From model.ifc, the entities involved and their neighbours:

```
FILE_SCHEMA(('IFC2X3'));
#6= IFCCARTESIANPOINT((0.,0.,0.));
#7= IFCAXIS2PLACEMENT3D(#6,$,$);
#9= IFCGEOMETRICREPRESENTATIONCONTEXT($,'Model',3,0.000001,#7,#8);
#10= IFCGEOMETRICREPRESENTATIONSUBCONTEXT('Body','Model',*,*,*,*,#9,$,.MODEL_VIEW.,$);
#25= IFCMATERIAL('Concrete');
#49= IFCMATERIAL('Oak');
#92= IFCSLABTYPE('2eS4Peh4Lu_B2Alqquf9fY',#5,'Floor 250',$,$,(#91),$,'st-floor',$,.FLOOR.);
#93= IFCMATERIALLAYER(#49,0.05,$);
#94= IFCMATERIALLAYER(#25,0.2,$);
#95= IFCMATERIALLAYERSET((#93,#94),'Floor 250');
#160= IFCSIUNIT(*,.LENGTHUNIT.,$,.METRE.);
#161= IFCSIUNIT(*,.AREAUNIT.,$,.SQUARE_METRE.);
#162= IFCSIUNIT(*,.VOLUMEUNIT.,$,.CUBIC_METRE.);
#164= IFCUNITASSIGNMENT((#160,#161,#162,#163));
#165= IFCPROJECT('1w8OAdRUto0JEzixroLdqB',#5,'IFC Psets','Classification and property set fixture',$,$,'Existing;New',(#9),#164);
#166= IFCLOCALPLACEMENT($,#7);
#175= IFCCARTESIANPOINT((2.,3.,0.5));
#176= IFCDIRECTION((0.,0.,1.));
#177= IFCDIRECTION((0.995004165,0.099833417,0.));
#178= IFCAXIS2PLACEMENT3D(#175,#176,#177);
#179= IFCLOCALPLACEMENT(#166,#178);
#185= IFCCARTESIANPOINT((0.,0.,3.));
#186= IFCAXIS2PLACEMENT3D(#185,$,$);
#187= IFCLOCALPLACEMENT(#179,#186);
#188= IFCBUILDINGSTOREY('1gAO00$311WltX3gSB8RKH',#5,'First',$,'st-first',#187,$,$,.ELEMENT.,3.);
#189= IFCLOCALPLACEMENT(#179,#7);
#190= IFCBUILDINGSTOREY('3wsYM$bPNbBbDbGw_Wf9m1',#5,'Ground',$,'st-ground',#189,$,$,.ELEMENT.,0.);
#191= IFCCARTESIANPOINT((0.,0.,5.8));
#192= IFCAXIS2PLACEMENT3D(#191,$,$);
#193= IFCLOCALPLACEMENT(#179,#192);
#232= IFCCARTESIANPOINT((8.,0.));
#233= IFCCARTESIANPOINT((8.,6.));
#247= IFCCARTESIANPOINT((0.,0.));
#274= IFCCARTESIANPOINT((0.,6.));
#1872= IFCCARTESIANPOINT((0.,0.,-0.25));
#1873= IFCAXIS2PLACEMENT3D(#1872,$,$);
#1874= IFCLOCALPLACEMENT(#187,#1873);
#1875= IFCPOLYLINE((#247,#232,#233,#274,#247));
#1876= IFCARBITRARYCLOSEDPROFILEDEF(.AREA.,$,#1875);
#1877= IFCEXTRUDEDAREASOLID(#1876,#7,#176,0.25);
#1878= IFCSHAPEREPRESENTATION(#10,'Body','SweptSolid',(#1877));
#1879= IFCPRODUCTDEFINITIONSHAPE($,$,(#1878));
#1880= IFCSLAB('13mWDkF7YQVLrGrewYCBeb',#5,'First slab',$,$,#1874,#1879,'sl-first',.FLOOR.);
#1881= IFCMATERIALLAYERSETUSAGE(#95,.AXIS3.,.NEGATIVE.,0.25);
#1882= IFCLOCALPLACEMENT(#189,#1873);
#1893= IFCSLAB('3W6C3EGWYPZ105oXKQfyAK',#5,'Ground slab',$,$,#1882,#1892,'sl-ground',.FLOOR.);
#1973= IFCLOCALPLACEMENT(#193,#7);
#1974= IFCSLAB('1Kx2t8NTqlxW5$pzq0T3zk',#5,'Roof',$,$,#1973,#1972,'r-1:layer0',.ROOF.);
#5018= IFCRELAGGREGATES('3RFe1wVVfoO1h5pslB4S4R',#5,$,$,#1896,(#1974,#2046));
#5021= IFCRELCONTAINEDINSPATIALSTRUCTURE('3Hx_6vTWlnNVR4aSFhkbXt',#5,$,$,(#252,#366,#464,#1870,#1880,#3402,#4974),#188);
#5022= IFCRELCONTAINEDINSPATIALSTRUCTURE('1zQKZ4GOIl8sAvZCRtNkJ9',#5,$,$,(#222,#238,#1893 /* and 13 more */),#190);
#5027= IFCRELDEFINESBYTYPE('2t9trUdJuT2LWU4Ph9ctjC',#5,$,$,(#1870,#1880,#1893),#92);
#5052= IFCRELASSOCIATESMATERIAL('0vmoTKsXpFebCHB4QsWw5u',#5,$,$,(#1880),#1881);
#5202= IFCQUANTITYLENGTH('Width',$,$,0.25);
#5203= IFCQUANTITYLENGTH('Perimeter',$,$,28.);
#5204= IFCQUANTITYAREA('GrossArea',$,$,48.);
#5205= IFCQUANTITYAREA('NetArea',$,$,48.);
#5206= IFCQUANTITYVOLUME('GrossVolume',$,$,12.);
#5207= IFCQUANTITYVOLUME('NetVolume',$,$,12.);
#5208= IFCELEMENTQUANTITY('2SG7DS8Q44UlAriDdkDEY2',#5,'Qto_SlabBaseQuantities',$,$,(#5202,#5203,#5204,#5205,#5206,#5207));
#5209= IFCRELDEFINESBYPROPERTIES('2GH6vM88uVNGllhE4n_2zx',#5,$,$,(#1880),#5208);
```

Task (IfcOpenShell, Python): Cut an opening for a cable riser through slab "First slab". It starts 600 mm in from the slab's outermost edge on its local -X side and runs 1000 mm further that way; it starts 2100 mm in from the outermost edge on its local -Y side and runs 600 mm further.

```python
import numpy as np
import ifcopenshell
import ifcopenshell.api.feature
import ifcopenshell.api.geometry
import ifcopenshell.api.pset
import ifcopenshell.api.root
import ifcopenshell.geom
import ifcopenshell.util.element
import ifcopenshell.util.placement
import ifcopenshell.util.representation
import ifcopenshell.util.shape
import ifcopenshell.util.unit

model = ifcopenshell.open("model.ifc")
unit_scale = ifcopenshell.util.unit.calculate_unit_scale(model)
area_scale = ifcopenshell.util.unit.calculate_unit_scale(model, "AREAUNIT")
volume_scale = ifcopenshell.util.unit.calculate_unit_scale(model, "VOLUMEUNIT")
settings = ifcopenshell.geom.settings()


def volume(element):
    """Net volume in cubic metres, openings subtracted."""
    shape = ifcopenshell.geom.create_shape(settings, element)
    return ifcopenshell.util.shape.get_volume(shape.geometry)


slab = model.by_id(1880)
before = volume(slab)

# Extent in the slab's own axes, in metres. The edges named are its -X and -Y sides.
slab_shape = ifcopenshell.geom.create_shape(settings, slab)
vertices = ifcopenshell.util.shape.get_vertices(slab_shape.geometry)
x_min, y_min, bottom = vertices.min(axis=0)
top = vertices[:, 2].max()

opening = ifcopenshell.api.root.create_entity(model, ifc_class="IfcOpeningElement", name="Cable riser opening")
context = ifcopenshell.util.representation.get_context(model, "Model", "Body", "MODEL_VIEW")
width, depth = 1, 0.6
outline = [(0.0, 0.0), (width, 0.0), (width, depth), (0.0, depth), (0.0, 0.0)]
# Overshoot both faces by 50 mm so the cut is clean.
shape = ifcopenshell.api.geometry.add_slab_representation(
    model, context=context, depth=top - bottom + 0.1, polyline=outline
)
ifcopenshell.api.geometry.assign_representation(model, product=opening, representation=shape)

matrix = ifcopenshell.util.placement.get_local_placement(slab.ObjectPlacement)
matrix[:, 3] = matrix @ np.append(np.array([x_min + 0.6, y_min + 2.1, bottom - 0.05]) / unit_scale, 1.0)
ifcopenshell.api.geometry.edit_object_placement(model, product=opening, matrix=matrix, is_si=False)
ifcopenshell.api.feature.add_feature(model, feature=opening, element=slab)

after = volume(slab)

# Update the slab's stored quantities.
qto = model.by_id(ifcopenshell.util.element.get_pset(slab, "Qto_SlabBaseQuantities", should_inherit=False)["id"])
ifcopenshell.api.pset.edit_qto(model, qto=qto, properties={
    "NetArea": after / (top - bottom) / area_scale,
    "NetVolume": after / volume_scale,
})

print(f"slab volume {before:.3f} -> {after:.3f} m3")

model.write("model_v2.ifc")
```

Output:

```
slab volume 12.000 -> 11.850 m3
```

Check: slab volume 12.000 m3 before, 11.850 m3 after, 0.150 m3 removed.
